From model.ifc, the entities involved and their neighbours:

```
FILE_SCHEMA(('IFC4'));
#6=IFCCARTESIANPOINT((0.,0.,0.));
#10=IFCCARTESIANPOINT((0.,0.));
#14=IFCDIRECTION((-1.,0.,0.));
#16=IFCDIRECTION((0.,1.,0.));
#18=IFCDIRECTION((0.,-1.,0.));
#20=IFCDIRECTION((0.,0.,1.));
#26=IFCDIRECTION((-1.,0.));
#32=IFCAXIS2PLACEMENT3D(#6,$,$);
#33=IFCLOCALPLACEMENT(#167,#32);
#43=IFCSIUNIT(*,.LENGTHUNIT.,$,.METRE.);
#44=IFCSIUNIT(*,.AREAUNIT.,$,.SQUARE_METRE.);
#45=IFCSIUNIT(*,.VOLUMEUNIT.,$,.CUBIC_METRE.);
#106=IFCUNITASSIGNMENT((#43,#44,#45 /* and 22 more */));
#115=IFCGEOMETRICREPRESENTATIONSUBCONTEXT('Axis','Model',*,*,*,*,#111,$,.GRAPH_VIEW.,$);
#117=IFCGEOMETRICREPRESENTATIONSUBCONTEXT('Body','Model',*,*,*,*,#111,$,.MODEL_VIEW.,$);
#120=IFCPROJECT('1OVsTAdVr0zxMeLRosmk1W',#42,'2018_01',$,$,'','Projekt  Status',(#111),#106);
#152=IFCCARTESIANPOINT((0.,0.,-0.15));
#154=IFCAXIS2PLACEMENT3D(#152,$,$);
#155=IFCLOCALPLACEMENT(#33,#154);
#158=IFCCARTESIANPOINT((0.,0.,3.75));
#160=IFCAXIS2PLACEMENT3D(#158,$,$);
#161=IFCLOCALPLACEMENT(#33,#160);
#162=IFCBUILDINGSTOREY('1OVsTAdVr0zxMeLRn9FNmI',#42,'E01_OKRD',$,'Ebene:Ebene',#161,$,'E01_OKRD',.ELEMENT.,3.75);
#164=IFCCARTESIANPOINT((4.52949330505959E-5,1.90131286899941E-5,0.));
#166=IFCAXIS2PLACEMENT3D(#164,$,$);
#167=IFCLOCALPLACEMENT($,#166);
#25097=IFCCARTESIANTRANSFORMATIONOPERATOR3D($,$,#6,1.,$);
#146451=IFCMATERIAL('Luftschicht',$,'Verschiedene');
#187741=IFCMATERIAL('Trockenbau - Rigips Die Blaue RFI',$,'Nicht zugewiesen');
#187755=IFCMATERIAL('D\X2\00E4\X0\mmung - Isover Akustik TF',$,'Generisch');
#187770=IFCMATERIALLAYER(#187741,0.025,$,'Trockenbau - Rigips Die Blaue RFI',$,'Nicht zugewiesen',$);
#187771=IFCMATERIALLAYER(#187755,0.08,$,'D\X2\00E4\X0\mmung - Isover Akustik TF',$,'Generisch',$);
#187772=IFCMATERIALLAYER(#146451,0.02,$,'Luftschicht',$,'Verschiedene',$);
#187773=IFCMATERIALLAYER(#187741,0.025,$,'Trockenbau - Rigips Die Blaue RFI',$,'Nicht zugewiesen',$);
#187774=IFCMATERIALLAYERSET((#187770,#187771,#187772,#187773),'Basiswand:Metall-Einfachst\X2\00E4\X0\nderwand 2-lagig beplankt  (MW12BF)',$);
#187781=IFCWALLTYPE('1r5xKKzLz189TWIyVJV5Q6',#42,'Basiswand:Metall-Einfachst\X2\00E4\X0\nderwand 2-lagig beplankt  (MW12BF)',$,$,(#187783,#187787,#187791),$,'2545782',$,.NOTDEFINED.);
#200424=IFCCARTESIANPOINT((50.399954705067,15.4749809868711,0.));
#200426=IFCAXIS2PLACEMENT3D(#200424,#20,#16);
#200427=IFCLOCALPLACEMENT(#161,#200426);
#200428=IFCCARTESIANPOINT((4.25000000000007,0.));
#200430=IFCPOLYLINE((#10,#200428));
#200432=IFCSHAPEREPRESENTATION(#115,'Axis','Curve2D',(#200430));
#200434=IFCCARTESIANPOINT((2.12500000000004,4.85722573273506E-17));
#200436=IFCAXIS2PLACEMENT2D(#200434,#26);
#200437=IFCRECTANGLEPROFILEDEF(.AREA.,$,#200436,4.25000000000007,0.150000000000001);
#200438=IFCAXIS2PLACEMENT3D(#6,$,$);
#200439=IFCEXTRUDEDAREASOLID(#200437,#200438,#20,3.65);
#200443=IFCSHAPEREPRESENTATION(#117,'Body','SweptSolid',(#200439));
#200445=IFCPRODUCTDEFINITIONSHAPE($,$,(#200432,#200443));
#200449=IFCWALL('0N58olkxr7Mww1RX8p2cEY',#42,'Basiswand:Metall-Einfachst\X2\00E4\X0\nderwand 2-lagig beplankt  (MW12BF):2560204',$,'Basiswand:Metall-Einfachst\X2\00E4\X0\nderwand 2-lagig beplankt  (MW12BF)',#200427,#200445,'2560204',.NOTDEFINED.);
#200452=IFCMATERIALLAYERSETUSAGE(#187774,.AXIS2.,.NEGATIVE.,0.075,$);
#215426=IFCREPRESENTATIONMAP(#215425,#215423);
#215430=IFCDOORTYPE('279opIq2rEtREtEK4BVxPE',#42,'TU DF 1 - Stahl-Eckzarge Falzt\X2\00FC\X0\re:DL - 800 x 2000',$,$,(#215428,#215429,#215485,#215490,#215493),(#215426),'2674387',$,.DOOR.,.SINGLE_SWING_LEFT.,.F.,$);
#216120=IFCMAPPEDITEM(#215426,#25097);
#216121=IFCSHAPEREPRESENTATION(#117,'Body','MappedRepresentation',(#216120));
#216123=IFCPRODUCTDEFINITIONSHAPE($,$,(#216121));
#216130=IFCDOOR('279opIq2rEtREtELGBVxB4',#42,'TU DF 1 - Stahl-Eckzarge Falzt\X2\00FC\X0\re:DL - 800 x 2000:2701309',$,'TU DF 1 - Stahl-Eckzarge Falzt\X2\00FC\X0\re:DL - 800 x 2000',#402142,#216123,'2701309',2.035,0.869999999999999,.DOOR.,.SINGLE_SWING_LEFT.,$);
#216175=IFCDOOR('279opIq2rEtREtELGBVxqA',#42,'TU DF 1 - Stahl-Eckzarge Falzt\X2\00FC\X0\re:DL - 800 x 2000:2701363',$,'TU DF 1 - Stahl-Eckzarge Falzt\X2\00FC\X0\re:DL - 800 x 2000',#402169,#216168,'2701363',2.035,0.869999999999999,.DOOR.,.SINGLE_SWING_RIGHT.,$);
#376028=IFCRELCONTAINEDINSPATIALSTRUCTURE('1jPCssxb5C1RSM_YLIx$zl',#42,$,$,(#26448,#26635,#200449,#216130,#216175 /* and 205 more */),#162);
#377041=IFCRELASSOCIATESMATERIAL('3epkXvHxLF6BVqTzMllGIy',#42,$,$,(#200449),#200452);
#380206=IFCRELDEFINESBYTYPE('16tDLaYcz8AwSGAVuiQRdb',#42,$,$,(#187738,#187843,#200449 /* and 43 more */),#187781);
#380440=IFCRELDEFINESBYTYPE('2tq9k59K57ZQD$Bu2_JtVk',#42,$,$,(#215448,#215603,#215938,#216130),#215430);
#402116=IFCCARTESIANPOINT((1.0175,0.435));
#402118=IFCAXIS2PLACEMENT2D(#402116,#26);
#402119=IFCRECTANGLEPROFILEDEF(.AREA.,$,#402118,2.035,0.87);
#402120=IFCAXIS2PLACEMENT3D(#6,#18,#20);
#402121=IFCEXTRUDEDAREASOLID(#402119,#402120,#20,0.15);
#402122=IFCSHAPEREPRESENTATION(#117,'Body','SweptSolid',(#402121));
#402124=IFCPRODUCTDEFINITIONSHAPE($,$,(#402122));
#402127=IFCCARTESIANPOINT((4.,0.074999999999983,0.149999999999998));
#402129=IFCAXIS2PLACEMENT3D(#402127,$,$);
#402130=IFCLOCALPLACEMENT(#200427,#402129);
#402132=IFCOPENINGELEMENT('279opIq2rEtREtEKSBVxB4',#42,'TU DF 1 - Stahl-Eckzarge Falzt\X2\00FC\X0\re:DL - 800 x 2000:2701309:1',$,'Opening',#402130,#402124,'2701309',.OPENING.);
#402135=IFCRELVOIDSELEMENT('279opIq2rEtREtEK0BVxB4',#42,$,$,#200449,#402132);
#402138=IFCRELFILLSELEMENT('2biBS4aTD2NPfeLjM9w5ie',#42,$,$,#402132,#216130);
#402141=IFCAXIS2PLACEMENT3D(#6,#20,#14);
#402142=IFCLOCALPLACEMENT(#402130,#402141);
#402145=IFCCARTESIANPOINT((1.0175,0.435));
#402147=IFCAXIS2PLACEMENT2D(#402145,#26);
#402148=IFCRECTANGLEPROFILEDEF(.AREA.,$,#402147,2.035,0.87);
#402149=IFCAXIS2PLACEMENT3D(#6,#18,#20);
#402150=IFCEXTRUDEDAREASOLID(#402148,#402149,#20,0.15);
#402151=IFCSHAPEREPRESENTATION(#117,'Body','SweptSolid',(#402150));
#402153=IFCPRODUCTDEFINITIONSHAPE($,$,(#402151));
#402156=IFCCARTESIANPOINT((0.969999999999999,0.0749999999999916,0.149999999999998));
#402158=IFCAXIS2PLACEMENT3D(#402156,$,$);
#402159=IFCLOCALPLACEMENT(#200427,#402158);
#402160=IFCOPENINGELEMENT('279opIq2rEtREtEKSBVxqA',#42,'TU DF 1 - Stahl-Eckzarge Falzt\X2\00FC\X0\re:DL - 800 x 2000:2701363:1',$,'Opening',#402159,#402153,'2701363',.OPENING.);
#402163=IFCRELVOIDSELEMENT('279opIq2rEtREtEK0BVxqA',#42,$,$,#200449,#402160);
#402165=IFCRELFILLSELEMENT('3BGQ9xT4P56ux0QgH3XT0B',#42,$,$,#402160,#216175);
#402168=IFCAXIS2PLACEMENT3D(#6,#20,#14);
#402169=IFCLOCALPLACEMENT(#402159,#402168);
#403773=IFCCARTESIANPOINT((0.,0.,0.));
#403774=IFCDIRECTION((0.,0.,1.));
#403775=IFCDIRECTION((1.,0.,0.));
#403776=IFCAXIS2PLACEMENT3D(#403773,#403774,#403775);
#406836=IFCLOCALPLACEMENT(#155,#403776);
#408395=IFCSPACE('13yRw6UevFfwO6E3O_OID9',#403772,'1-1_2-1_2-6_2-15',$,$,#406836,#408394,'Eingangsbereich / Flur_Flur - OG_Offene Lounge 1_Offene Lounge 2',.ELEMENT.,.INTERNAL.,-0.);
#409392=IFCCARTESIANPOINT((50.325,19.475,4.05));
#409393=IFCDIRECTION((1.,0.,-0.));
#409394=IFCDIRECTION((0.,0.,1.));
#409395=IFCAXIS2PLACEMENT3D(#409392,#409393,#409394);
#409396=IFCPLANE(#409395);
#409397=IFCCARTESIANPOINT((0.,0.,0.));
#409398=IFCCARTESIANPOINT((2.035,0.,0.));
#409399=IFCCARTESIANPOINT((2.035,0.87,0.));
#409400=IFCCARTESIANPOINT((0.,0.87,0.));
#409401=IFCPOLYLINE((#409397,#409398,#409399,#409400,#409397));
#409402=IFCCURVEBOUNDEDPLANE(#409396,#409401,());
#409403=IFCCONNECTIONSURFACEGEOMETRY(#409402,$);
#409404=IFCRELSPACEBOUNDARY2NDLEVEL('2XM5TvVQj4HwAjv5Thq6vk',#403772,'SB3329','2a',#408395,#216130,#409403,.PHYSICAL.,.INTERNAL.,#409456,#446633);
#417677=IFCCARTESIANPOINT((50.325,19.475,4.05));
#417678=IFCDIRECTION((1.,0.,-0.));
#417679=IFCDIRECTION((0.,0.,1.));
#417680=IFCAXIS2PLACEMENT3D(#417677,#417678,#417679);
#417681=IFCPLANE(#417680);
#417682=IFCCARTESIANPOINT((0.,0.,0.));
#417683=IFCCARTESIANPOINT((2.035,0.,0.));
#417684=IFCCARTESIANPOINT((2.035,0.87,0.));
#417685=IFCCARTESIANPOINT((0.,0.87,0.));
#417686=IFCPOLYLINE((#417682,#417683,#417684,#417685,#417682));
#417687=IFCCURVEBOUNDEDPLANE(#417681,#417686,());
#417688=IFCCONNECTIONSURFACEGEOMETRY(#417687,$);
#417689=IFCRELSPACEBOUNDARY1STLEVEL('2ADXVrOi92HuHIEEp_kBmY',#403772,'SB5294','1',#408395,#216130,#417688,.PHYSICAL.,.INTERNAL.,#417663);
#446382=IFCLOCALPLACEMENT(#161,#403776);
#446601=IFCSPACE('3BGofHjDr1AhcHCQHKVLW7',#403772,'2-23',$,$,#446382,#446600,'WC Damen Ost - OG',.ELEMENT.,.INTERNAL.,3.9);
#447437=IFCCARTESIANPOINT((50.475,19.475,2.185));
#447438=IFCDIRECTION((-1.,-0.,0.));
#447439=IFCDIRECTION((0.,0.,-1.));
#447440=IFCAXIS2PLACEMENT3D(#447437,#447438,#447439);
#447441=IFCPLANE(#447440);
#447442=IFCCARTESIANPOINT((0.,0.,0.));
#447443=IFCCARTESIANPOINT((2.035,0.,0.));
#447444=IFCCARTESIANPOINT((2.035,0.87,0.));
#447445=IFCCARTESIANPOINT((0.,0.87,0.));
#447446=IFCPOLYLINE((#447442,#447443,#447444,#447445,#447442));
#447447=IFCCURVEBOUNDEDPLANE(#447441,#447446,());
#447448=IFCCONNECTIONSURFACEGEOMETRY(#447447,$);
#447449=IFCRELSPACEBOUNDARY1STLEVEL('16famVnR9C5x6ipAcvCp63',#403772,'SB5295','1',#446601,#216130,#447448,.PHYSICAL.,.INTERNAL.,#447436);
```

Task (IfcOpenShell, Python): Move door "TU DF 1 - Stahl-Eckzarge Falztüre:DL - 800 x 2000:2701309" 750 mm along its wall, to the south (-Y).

```python
import numpy as np
import ifcopenshell
import ifcopenshell.api.geometry
import ifcopenshell.util.placement
import ifcopenshell.util.unit

model = ifcopenshell.open("model.ifc")
unit_scale = ifcopenshell.util.unit.calculate_unit_scale(model)

door = model.by_guid("279opIq2rEtREtELGBVxB4")
opening = door.FillsVoids[0].RelatingOpeningElement
wall = opening.VoidsElements[0].RelatingBuildingElement

wall_matrix = ifcopenshell.util.placement.get_local_placement(wall.ObjectPlacement)
shift = wall_matrix[:3, 0] * -0.75 / unit_scale
before = ifcopenshell.util.placement.get_local_placement(door.ObjectPlacement)[:3, 3].copy()

# The door is placed relative to its opening, so it follows when the opening moves.
matrix = ifcopenshell.util.placement.get_local_placement(opening.ObjectPlacement)
matrix[:3, 3] += shift
ifcopenshell.api.geometry.edit_object_placement(
    model, product=opening, matrix=matrix, is_si=False, should_transform_children=True
)

# Space boundary surfaces are stored in each space's coordinates; move them too.
for rel in door.ProvidesBoundaries:
    if not rel.ConnectionGeometry:
        continue
    surface = rel.ConnectionGeometry.SurfaceOnRelatingElement.BasisSurface
    space_matrix = ifcopenshell.util.placement.get_local_placement(rel.RelatingSpace.ObjectPlacement)
    point = np.array(surface.Position.Location.Coordinates) + space_matrix[:3, :3].T @ shift
    surface.Position = model.createIfcAxis2Placement3D(
        model.createIfcCartesianPoint(point.tolist()), surface.Position.Axis, surface.Position.RefDirection
    )

after = ifcopenshell.util.placement.get_local_placement(door.ObjectPlacement)[:3, 3]
print("door moved by", (after - before).round(3) + 0.0)

model.write("model_edited.ifc")
```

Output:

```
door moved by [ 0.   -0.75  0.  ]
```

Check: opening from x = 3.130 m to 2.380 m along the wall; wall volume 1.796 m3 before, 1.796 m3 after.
